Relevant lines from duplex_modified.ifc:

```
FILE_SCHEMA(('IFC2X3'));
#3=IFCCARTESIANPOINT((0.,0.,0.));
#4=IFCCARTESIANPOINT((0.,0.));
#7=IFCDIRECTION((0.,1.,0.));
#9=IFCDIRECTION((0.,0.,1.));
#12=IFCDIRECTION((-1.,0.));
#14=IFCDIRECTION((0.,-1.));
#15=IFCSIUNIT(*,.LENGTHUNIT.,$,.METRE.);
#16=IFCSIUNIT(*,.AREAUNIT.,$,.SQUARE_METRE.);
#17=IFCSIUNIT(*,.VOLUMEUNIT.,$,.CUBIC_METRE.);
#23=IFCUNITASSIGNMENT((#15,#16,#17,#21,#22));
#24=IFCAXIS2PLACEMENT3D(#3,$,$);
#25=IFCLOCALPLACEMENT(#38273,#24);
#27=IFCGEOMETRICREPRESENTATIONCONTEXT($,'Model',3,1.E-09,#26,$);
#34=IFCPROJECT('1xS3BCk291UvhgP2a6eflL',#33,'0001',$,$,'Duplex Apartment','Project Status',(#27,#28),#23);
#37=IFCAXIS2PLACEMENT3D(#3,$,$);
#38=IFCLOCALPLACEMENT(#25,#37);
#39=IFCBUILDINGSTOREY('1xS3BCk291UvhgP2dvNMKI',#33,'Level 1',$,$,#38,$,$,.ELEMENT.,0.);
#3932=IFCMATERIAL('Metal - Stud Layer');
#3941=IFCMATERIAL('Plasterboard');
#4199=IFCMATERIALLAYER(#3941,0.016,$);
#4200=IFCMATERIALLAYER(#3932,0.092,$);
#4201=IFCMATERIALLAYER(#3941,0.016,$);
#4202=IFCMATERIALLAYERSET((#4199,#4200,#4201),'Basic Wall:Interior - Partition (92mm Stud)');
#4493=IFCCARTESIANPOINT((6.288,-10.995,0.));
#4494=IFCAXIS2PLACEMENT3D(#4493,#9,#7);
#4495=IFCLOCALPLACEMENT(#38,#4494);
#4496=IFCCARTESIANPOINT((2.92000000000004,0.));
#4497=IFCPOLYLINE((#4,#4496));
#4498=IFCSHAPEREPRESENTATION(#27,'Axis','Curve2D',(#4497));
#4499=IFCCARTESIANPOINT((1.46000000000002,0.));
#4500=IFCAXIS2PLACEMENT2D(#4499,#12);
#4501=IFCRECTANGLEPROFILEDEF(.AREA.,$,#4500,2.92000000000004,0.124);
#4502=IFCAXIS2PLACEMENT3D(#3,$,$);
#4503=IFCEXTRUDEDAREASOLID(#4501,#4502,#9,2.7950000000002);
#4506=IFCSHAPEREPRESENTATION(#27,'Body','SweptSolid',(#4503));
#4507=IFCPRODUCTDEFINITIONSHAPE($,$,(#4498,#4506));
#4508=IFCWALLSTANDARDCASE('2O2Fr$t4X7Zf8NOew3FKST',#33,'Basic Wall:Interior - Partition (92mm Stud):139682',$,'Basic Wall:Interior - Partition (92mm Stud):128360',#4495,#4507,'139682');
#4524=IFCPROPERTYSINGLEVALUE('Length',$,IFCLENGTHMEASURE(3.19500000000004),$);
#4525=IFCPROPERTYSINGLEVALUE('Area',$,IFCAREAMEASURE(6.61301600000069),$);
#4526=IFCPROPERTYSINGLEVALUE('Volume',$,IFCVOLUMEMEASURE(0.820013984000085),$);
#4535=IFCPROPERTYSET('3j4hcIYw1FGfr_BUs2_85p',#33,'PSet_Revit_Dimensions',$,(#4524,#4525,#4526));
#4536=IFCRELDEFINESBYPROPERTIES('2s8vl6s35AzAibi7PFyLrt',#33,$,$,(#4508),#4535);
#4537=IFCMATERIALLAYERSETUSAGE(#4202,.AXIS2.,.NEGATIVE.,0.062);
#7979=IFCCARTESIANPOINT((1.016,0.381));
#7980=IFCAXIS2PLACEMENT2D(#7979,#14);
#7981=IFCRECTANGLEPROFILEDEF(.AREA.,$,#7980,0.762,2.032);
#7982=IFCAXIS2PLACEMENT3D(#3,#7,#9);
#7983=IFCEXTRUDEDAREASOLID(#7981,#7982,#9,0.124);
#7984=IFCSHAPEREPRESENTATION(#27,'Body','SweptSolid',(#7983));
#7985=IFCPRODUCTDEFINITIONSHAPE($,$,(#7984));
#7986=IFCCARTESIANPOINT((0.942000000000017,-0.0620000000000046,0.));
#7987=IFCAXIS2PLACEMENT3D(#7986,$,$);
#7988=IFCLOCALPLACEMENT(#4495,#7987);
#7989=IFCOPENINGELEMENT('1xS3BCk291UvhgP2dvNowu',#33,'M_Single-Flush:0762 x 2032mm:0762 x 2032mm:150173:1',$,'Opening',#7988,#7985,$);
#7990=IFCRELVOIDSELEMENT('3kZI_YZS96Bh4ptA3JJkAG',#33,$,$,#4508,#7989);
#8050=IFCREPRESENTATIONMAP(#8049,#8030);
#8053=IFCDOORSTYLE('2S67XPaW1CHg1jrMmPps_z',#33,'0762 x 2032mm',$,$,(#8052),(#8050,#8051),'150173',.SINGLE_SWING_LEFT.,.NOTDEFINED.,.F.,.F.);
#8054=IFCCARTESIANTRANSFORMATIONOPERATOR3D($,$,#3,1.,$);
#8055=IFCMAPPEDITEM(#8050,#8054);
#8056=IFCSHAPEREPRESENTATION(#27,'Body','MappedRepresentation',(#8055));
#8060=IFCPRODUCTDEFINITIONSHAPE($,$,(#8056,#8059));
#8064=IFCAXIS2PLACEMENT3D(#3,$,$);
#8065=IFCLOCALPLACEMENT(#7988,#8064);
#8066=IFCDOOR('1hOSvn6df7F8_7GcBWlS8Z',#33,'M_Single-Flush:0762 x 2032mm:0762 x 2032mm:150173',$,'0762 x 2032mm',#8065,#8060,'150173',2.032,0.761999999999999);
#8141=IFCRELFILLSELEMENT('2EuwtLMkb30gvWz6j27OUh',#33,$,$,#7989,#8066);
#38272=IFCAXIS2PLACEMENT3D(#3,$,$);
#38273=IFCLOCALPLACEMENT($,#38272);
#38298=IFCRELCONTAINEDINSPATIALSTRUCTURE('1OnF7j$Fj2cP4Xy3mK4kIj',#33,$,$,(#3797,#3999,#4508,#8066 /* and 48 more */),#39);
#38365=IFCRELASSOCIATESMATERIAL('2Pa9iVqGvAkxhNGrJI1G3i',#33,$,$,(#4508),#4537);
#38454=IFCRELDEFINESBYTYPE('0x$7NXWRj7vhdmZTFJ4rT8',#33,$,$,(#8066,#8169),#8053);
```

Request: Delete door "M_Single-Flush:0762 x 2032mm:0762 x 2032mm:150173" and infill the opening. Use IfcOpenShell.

```python
import ifcopenshell
import ifcopenshell.api.feature
import ifcopenshell.api.pset
import ifcopenshell.api.root
import ifcopenshell.geom
import ifcopenshell.util.element
import ifcopenshell.util.shape
import ifcopenshell.util.unit

model = ifcopenshell.open("duplex_modified.ifc")
area_scale = ifcopenshell.util.unit.calculate_unit_scale(model, "AREAUNIT")
volume_scale = ifcopenshell.util.unit.calculate_unit_scale(model, "VOLUMEUNIT")
settings = ifcopenshell.geom.settings()


def volume(element):
    """Net volume in cubic metres, openings subtracted."""
    shape = ifcopenshell.geom.create_shape(settings, element)
    return ifcopenshell.util.shape.get_volume(shape.geometry)


door = model.by_guid("1hOSvn6df7F8_7GcBWlS8Z")
opening = door.FillsVoids[0].RelatingOpeningElement
wall = opening.VoidsElements[0].RelatingBuildingElement
before = volume(wall)

ifcopenshell.api.root.remove_product(model, product=door)
ifcopenshell.api.feature.remove_feature(model, feature=opening)

after = volume(wall)
thickness = 0.124  # wall thickness in metres

# Update the wall's stored quantities.
pset = model.by_id(ifcopenshell.util.element.get_pset(wall, "PSet_Revit_Dimensions", should_inherit=False)["id"])
ifcopenshell.api.pset.edit_pset(model, pset=pset, properties={
    "Area": model.create_entity("IfcAreaMeasure", after / thickness / area_scale),
    "Volume": model.create_entity("IfcVolumeMeasure", after / volume_scale),
})

print(f"wall volume {before:.3f} -> {after:.3f} m3")

model.write("duplex_modified-out.ifc")
```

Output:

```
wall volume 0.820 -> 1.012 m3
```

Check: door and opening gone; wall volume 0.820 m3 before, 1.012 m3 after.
